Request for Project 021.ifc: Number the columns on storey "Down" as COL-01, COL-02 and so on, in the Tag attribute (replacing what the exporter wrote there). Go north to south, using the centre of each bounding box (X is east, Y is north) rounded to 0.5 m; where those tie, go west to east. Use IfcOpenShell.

First a look at what the model holds.

```python
import ifcopenshell
import ifcopenshell.util.element
import ifcopenshell.util.placement

model = ifcopenshell.open("Project 021.ifc")
print(model.schema)
storey = next(s for s in model.by_type("IfcBuildingStorey") if s.Name == "Down")
columns = [e for e in ifcopenshell.util.element.get_decomposition(storey) if e.is_a("IfcColumn")]
for e in sorted(columns, key=lambda e: e.id()):
    origin = ifcopenshell.util.placement.get_local_placement(e.ObjectPlacement)[:3, 3]
    print(e.id(), e.Tag, e.Name, origin.round(2) + 0.0, sep=" | ")
```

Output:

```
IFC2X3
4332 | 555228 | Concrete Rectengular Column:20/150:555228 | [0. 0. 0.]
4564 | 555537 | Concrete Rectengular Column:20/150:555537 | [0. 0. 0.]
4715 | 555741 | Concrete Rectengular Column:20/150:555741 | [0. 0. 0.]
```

```python
import ifcopenshell
import ifcopenshell.geom
import ifcopenshell.util.element
import ifcopenshell.util.shape

model = ifcopenshell.open("Project 021.ifc")
settings = ifcopenshell.geom.settings()
settings.set("use-world-coords", True)


def centre(element):
    shape = ifcopenshell.geom.create_shape(settings, element)
    return ifcopenshell.util.shape.get_bbox_centroid(shape.geometry)


storey = next(s for s in model.by_type("IfcBuildingStorey") if s.Name == "Down")
columns = [e for e in ifcopenshell.util.element.get_decomposition(storey) if e.is_a("IfcColumn")]

# Insertion points can sit at a corner or the storey origin, so sort by the geometry (in metres).
centres = {e: centre(e) for e in columns}
columns.sort(key=lambda e: (-round(centres[e][1] / 0.5), centres[e][0]))

for i, e in enumerate(columns, start=1):
    number = f"COL-{i:02d}"
    e.Tag = number
    print(e.id(), number)

model.write("Project 021_rev.ifc")
```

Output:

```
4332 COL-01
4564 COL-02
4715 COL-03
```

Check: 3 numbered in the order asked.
